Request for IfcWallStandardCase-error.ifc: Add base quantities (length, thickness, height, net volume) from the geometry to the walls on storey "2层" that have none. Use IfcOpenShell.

First a look at what the model holds.

```python
import ifcopenshell
import ifcopenshell.util.element
import ifcopenshell.util.unit

model = ifcopenshell.open("IfcWallStandardCase-error.ifc")
print(model.schema)
for unit_type in ("LENGTHUNIT", "AREAUNIT", "VOLUMEUNIT"):
    print(unit_type, ifcopenshell.util.unit.calculate_unit_scale(model, unit_type))
storey = next(s for s in model.by_type("IfcBuildingStorey") if s.Name == "2层")
walls = [e for e in ifcopenshell.util.element.get_decomposition(storey) if e.is_a("IfcWall")]
for e in sorted(walls, key=lambda e: e.id()):
    print(e.id(), e.is_a(), e.Name, list(ifcopenshell.util.element.get_psets(e, qtos_only=True)), sep=" | ")
```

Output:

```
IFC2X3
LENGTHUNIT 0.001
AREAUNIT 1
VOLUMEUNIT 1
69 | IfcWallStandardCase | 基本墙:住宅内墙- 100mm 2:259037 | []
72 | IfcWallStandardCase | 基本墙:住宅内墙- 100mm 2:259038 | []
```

```python
import ifcopenshell
import ifcopenshell.api.pset
import ifcopenshell.geom
import ifcopenshell.util.element
import ifcopenshell.util.shape
import ifcopenshell.util.unit

model = ifcopenshell.open("IfcWallStandardCase-error.ifc")
unit_scale = ifcopenshell.util.unit.calculate_unit_scale(model)
volume_scale = ifcopenshell.util.unit.calculate_unit_scale(model, "VOLUMEUNIT")
settings = ifcopenshell.geom.settings()

storey = next(s for s in model.by_type("IfcBuildingStorey") if s.Name == "2层")
walls = [e for e in ifcopenshell.util.element.get_decomposition(storey) if e.is_a("IfcWall")]

for e in sorted(walls, key=lambda e: e.id()):
    if ifcopenshell.util.element.get_psets(e, qtos_only=True, should_inherit=False):
        continue
    # Geometry comes back in metres, in the element's own axes.
    shape = ifcopenshell.geom.create_shape(settings, e)
    values = {
        "Length": ifcopenshell.util.shape.get_x(shape.geometry) / unit_scale,
        "Width": ifcopenshell.util.shape.get_y(shape.geometry) / unit_scale,
        "Height": ifcopenshell.util.shape.get_z(shape.geometry) / unit_scale,
        "NetVolume": ifcopenshell.util.shape.get_volume(shape.geometry) / volume_scale,
    }
    qto = ifcopenshell.api.pset.add_qto(model, product=e, name="BaseQuantities")
    ifcopenshell.api.pset.edit_qto(model, qto=qto, properties=values)
    print(e.id(), {k: round(v, 3) for k, v in values.items()})

model.write("IfcWallStandardCase-error_edited.ifc")
```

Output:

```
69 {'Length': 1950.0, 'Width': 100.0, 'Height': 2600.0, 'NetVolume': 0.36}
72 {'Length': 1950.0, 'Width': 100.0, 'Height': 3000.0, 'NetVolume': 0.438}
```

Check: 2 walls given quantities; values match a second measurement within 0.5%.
